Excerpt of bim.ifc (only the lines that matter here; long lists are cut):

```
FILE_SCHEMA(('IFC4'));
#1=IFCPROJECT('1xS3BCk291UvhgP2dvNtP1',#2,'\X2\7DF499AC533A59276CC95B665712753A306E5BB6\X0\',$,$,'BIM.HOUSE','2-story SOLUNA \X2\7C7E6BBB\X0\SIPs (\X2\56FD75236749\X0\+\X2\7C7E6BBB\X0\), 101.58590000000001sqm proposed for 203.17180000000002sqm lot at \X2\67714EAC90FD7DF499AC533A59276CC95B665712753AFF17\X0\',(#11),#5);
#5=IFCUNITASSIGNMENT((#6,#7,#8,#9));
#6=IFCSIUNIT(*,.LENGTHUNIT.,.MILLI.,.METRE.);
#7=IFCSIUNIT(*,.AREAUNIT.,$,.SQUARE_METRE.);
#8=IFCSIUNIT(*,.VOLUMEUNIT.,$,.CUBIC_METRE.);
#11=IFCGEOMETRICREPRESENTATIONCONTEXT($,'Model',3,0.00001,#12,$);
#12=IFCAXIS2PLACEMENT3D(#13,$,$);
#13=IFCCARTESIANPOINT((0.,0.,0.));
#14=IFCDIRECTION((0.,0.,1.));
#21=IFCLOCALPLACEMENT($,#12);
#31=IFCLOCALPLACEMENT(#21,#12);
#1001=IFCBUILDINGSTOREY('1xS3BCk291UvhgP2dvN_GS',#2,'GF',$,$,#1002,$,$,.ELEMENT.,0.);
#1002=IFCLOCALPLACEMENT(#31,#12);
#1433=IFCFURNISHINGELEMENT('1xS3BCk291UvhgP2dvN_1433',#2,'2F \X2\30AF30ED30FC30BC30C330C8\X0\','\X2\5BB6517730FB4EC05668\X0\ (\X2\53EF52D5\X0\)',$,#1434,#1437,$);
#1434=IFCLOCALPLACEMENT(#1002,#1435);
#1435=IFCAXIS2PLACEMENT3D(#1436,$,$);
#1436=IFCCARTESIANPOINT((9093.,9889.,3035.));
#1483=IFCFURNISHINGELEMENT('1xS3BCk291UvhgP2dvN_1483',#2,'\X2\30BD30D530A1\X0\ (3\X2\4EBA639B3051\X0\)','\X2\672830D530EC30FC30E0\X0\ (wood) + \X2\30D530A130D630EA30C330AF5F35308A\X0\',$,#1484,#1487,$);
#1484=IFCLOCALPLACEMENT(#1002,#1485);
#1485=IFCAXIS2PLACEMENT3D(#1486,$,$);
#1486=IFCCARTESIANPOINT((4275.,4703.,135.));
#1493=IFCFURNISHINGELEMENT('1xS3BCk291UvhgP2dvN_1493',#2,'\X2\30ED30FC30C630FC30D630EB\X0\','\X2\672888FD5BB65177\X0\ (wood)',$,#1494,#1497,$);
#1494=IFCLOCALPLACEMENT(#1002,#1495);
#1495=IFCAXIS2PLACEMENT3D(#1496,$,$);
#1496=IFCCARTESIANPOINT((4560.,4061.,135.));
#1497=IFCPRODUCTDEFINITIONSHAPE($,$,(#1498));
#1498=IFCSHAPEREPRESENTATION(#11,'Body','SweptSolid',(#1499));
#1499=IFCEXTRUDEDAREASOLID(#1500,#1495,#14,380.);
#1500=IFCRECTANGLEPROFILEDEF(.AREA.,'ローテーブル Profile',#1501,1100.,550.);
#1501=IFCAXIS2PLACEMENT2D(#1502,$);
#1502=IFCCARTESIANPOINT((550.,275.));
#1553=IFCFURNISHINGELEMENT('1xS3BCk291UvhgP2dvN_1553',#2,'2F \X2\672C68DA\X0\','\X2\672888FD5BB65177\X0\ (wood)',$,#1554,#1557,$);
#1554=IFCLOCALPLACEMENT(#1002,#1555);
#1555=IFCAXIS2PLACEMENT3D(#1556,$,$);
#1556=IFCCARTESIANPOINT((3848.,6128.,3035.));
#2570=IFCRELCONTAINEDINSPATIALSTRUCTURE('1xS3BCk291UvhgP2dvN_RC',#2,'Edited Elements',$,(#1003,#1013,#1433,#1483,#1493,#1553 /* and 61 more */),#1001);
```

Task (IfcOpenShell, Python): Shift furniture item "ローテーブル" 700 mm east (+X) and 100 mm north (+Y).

```python
import ifcopenshell
import ifcopenshell.api.geometry
import ifcopenshell.util.placement

model = ifcopenshell.open("bim.ifc")

item = model.by_id(1493)
matrix = ifcopenshell.util.placement.get_local_placement(item.ObjectPlacement)
matrix[0, 3] += 700.0
matrix[1, 3] += 100.0
ifcopenshell.api.geometry.edit_object_placement(model, product=item, matrix=matrix, is_si=False)

print(ifcopenshell.util.placement.get_local_placement(item.ObjectPlacement).round(3) + 0.0)

model.write("bim_edited.ifc")
```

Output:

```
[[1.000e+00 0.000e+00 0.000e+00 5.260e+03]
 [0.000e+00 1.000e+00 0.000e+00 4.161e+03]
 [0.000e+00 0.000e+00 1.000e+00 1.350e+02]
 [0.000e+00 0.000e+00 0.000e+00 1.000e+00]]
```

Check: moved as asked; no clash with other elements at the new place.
